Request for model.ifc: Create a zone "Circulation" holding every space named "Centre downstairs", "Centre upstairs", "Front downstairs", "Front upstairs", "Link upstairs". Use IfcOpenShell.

First a look at what the model holds.

```python
import ifcopenshell

model = ifcopenshell.open("model.ifc")
print(model.schema)
seen = {}
for space in model.by_type("IfcSpace"):
    seen[space.Name] = seen.get(space.Name, 0) + 1
for name, count in sorted(seen.items(), key=str):
    print(count, "x", name)
print("zones:", [z.Name for z in model.by_type("IfcZone")][:20])
```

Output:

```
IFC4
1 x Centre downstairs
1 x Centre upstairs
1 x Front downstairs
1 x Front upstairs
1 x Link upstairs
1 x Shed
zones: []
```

```python
import ifcopenshell
import ifcopenshell.api.group
import ifcopenshell.api.root

model = ifcopenshell.open("model.ifc")

names = {"Centre downstairs", "Centre upstairs", "Front downstairs", "Front upstairs", "Link upstairs"}
spaces = [s for s in model.by_type("IfcSpace") if s.Name in names]

zone = ifcopenshell.api.root.create_entity(model, ifc_class="IfcZone", name="Circulation")
ifcopenshell.api.group.assign_group(model, products=spaces, group=zone)
print(len(spaces), "spaces in", zone.Name)

model.write("model_rev.ifc")
```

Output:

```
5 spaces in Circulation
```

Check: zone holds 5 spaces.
